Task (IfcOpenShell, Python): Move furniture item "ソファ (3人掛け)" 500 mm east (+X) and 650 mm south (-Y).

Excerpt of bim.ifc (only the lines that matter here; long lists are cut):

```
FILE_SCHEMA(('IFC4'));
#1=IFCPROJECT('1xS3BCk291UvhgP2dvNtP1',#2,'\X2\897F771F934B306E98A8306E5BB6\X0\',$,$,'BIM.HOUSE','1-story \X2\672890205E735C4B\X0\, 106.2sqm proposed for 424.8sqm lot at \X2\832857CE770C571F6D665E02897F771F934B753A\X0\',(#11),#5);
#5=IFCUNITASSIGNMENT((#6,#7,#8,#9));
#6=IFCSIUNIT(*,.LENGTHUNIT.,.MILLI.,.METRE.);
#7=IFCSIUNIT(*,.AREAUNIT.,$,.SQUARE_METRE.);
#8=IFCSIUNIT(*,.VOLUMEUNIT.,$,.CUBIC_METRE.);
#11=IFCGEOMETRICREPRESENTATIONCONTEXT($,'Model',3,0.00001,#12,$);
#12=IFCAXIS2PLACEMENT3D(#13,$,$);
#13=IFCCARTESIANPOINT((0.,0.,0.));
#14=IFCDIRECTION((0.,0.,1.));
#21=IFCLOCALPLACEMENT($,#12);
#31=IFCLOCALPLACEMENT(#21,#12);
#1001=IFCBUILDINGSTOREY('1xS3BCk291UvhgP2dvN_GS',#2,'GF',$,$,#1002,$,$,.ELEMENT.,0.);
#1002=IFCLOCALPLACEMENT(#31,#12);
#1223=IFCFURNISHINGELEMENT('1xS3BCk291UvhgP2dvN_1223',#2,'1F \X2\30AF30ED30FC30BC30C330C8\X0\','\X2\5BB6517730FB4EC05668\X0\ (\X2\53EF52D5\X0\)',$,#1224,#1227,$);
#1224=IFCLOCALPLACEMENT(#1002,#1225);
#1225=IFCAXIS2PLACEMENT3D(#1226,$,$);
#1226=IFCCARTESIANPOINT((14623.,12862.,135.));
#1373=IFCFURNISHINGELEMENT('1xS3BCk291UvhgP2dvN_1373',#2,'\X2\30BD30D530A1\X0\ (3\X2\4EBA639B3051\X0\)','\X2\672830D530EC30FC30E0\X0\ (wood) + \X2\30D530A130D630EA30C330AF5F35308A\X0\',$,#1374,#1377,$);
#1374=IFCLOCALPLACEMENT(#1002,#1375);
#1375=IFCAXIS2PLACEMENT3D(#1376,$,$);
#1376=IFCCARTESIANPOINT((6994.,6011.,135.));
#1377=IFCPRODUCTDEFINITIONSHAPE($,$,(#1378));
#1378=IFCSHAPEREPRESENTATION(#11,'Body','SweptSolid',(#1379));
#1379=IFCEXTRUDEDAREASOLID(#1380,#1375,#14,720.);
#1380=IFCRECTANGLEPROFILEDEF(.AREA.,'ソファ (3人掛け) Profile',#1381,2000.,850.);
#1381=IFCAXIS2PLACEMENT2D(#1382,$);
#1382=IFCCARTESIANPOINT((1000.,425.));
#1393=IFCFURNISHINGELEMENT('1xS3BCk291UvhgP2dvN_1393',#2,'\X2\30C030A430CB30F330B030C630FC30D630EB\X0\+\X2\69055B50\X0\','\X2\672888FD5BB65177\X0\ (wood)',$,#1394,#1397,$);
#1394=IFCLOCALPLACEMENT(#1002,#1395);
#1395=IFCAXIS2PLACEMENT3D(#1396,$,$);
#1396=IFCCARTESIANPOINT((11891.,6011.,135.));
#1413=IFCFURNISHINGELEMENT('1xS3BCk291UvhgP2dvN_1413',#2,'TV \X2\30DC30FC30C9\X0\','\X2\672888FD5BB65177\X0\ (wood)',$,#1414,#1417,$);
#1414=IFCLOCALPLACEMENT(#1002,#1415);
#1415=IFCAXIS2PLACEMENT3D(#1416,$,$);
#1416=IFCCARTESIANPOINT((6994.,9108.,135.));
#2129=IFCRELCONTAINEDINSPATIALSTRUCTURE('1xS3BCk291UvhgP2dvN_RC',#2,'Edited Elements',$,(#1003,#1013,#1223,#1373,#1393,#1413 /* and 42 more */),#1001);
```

```python
import ifcopenshell
import ifcopenshell.api.geometry
import ifcopenshell.util.placement

model = ifcopenshell.open("bim.ifc")

item = model.by_id(1373)
matrix = ifcopenshell.util.placement.get_local_placement(item.ObjectPlacement)
matrix[0, 3] += 500.0
matrix[1, 3] -= 650.0
ifcopenshell.api.geometry.edit_object_placement(model, product=item, matrix=matrix, is_si=False)

print(ifcopenshell.util.placement.get_local_placement(item.ObjectPlacement).round(3) + 0.0)

model.write("bim_edited.ifc")
```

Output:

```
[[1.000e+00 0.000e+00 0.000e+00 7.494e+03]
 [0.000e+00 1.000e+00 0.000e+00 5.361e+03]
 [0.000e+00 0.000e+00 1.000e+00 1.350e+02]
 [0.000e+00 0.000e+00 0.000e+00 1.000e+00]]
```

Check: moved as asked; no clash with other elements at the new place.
